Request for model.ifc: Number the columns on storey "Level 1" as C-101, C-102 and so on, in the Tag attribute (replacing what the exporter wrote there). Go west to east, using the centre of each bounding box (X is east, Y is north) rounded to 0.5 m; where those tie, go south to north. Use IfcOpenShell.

First a look at what the model holds.

```python
import ifcopenshell
import ifcopenshell.util.element
import ifcopenshell.util.placement

model = ifcopenshell.open("model.ifc")
print(model.schema)
storey = next(s for s in model.by_type("IfcBuildingStorey") if s.Name == "Level 1")
columns = [e for e in ifcopenshell.util.element.get_decomposition(storey) if e.is_a("IfcColumn")]
for e in sorted(columns, key=lambda e: e.id()):
    origin = ifcopenshell.util.placement.get_local_placement(e.ObjectPlacement)[:3, 3]
    print(e.id(), e.Tag, e.Name, origin.round(2) + 0.0, sep=" | ")
```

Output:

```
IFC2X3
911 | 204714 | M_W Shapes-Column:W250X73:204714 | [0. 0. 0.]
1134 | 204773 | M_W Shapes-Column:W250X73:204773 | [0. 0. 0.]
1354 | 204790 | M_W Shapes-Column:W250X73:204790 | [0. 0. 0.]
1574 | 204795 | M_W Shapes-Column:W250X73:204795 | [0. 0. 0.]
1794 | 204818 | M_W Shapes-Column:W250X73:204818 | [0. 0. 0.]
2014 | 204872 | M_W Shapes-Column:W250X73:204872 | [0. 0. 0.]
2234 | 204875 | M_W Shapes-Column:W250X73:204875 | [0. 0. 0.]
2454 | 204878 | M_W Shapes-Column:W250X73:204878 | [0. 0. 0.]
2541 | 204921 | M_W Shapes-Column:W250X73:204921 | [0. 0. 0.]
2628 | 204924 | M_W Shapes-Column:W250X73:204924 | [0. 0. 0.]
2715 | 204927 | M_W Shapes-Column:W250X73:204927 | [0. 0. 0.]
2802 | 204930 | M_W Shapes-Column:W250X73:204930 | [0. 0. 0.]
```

```python
import ifcopenshell
import ifcopenshell.geom
import ifcopenshell.util.element
import ifcopenshell.util.shape

model = ifcopenshell.open("model.ifc")
settings = ifcopenshell.geom.settings()
settings.set("use-world-coords", True)


def centre(element):
    shape = ifcopenshell.geom.create_shape(settings, element)
    return ifcopenshell.util.shape.get_bbox_centroid(shape.geometry)


storey = next(s for s in model.by_type("IfcBuildingStorey") if s.Name == "Level 1")
columns = [e for e in ifcopenshell.util.element.get_decomposition(storey) if e.is_a("IfcColumn")]

# Insertion points can sit at a corner or the storey origin, so sort by the geometry (in metres).
centres = {e: centre(e) for e in columns}
columns.sort(key=lambda e: (round(centres[e][0] / 0.5), centres[e][1]))

for i, e in enumerate(columns, start=1):
    number = f"C-1{i:02d}"
    e.Tag = number
    print(e.id(), number)

model.write("model-out.ifc")
```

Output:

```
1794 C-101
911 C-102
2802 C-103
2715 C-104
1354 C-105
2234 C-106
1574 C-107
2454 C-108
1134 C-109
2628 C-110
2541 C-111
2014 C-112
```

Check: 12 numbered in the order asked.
